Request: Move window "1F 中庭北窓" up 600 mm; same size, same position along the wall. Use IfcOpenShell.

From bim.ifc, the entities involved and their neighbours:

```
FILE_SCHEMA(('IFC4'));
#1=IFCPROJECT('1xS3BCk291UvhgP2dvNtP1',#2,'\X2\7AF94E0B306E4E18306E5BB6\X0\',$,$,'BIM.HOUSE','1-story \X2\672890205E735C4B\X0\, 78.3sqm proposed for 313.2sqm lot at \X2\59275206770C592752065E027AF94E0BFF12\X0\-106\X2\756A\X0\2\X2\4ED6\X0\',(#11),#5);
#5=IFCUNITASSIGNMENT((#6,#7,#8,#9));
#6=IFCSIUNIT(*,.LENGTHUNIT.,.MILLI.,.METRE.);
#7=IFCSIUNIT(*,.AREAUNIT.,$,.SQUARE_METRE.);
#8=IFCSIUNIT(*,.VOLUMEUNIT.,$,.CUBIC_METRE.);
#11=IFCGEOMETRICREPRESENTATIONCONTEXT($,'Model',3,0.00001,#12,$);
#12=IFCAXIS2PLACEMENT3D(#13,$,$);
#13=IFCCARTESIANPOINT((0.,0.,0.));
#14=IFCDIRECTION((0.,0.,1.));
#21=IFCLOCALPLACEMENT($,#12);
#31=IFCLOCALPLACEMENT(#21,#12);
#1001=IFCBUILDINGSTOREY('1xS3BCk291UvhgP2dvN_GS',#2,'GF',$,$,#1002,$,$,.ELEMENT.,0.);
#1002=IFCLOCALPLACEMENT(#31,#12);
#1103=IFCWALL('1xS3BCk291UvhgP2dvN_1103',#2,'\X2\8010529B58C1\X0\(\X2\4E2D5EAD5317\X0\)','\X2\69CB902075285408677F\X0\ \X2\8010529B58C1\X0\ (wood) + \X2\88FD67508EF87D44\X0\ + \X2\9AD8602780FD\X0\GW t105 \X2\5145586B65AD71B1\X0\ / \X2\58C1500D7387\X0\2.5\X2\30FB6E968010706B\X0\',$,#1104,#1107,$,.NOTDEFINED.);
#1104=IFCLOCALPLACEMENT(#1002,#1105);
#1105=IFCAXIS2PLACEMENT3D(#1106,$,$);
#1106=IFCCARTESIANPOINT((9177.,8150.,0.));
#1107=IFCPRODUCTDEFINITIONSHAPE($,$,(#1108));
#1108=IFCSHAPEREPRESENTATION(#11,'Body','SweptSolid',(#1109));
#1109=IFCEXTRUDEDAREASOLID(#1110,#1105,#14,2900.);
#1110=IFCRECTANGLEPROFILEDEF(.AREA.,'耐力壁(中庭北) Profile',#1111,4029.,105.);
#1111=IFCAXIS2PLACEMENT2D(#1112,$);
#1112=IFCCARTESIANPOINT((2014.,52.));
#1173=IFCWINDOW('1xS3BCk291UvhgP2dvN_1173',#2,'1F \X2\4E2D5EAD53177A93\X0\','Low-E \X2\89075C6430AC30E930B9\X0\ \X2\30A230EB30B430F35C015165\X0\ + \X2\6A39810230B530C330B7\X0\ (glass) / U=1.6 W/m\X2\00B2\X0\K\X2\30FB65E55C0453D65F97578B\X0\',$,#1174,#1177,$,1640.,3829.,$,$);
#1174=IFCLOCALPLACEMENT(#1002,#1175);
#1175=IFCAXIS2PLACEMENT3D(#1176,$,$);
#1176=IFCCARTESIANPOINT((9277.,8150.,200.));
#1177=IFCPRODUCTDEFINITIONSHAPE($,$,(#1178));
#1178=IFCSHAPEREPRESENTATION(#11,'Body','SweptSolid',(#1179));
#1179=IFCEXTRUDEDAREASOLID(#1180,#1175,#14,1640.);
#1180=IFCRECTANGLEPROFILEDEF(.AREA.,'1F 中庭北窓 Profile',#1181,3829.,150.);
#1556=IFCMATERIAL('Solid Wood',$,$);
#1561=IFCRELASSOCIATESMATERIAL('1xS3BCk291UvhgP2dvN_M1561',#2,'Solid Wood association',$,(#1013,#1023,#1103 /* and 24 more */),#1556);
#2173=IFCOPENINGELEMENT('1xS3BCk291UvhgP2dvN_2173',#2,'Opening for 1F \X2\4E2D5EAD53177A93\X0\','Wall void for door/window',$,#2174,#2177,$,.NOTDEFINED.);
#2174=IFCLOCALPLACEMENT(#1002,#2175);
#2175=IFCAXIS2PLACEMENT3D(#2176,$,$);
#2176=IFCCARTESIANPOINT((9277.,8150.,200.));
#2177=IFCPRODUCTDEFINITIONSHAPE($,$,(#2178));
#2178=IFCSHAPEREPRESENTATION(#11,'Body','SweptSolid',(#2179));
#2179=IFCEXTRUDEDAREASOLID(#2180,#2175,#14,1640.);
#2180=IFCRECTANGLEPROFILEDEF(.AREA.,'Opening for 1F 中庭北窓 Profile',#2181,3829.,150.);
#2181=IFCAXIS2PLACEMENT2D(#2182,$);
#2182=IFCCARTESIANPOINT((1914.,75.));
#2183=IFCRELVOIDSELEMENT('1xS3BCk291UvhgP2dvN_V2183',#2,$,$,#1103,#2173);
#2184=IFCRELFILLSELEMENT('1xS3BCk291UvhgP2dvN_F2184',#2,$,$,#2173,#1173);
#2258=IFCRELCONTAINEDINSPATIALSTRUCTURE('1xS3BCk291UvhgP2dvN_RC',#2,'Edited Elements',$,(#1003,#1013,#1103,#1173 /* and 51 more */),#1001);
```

```python
import numpy as np
import ifcopenshell
import ifcopenshell.api.geometry
import ifcopenshell.util.placement
import ifcopenshell.util.unit

model = ifcopenshell.open("bim.ifc")
unit_scale = ifcopenshell.util.unit.calculate_unit_scale(model)

window = model.by_guid("1xS3BCk291UvhgP2dvN_1173")
opening = window.FillsVoids[0].RelatingOpeningElement
dz = 0.6 / unit_scale

shift = np.array([0.0, 0.0, dz])
# The window is not placed relative to its opening, so move both.
for product in (opening, window):
    matrix = ifcopenshell.util.placement.get_local_placement(product.ObjectPlacement)
    matrix[:3, 3] += shift
    ifcopenshell.api.geometry.edit_object_placement(model, product=product, matrix=matrix, is_si=False)

print(f"moved by {dz * unit_scale:+.3f} m")

model.write("bim_edited.ifc")
```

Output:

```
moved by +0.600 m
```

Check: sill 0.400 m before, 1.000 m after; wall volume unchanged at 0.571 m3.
